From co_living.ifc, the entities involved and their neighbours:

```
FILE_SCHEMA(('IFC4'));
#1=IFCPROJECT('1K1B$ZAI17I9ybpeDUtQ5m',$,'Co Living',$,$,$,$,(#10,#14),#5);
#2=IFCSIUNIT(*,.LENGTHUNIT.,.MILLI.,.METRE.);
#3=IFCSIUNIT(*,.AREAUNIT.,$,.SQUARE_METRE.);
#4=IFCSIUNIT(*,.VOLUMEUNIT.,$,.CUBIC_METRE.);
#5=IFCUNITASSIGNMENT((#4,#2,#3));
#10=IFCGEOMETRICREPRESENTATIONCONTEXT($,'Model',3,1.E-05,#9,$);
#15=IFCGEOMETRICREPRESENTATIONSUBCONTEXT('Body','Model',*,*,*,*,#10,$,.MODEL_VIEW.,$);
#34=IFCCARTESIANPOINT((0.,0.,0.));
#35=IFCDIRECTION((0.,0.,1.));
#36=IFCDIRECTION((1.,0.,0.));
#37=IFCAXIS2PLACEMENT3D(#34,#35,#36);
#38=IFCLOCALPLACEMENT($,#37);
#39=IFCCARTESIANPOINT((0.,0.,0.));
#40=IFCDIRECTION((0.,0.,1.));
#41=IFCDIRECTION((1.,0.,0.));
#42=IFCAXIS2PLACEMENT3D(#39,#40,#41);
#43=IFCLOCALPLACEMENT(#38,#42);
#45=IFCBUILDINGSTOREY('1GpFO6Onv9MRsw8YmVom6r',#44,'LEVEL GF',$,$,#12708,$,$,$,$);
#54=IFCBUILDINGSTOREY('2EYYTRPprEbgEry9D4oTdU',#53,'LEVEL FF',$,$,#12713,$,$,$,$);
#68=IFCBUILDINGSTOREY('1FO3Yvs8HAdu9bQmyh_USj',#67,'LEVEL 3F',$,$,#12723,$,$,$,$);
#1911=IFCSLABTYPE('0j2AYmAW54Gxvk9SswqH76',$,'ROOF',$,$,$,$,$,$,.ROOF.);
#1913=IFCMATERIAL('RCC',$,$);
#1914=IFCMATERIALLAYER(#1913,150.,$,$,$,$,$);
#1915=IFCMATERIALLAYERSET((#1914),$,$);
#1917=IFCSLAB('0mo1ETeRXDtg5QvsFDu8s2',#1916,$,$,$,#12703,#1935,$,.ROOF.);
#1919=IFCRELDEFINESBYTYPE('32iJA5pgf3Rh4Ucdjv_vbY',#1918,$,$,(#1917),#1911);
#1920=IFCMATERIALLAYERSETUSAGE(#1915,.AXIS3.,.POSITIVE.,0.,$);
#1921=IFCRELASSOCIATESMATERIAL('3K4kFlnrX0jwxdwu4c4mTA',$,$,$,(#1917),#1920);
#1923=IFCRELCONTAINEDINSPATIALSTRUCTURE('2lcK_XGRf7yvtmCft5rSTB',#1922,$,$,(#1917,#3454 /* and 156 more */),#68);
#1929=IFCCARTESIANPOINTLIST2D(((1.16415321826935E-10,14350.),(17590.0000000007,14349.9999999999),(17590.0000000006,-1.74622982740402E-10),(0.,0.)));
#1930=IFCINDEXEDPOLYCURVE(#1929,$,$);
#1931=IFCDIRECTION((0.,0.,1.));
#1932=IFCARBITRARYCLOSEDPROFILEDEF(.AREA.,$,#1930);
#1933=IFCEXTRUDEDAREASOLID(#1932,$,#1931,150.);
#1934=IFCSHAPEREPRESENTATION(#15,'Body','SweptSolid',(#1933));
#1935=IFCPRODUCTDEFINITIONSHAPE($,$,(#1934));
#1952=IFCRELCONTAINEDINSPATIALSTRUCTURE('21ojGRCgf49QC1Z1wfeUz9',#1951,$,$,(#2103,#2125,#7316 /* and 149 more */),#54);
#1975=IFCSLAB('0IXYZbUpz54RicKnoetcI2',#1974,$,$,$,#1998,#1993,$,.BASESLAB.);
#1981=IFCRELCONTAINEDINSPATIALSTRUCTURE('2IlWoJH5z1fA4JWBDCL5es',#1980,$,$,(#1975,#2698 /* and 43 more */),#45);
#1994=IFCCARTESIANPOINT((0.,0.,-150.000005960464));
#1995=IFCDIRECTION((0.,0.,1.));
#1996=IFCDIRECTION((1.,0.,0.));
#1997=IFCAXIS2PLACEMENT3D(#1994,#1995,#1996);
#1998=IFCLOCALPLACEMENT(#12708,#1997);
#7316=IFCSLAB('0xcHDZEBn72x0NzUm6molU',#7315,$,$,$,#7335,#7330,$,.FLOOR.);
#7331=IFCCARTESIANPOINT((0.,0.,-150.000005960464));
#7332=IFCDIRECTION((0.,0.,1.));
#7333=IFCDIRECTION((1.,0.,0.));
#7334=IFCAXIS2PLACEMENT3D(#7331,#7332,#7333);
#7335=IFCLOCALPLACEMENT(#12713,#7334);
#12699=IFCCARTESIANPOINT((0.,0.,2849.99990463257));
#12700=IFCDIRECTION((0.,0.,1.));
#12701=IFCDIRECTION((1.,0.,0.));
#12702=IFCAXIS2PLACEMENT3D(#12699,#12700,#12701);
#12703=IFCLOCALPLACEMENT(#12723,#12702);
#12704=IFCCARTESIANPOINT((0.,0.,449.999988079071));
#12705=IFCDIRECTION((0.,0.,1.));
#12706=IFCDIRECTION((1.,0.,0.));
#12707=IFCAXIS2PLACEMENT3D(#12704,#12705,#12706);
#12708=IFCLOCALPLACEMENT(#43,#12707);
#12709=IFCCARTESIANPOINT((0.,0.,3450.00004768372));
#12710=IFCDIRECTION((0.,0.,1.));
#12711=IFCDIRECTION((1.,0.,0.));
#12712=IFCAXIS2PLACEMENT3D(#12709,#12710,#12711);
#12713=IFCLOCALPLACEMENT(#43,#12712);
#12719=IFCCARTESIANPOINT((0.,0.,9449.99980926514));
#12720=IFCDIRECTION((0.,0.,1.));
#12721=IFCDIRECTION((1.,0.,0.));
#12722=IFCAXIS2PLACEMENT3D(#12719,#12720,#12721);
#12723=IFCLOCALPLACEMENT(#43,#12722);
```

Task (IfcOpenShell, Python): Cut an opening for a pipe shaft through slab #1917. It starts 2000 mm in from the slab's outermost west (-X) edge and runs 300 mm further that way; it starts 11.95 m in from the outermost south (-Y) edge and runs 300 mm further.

```python
import numpy as np
import ifcopenshell
import ifcopenshell.api.feature
import ifcopenshell.api.geometry
import ifcopenshell.api.root
import ifcopenshell.geom
import ifcopenshell.util.placement
import ifcopenshell.util.representation
import ifcopenshell.util.shape
import ifcopenshell.util.unit

model = ifcopenshell.open("co_living.ifc")
unit_scale = ifcopenshell.util.unit.calculate_unit_scale(model)
settings = ifcopenshell.geom.settings()


def volume(element):
    """Net volume in cubic metres, openings subtracted."""
    shape = ifcopenshell.geom.create_shape(settings, element)
    return ifcopenshell.util.shape.get_volume(shape.geometry)


slab = model.by_id(1917)
before = volume(slab)

# Extent in the slab's own axes, in metres. The edges named are its -X and -Y sides.
slab_shape = ifcopenshell.geom.create_shape(settings, slab)
vertices = ifcopenshell.util.shape.get_vertices(slab_shape.geometry)
x_min, y_min, bottom = vertices.min(axis=0)
top = vertices[:, 2].max()

opening = ifcopenshell.api.root.create_entity(model, ifc_class="IfcOpeningElement", name="Pipe shaft opening", predefined_type="OPENING")
context = ifcopenshell.util.representation.get_context(model, "Model", "Body", "MODEL_VIEW")
width, depth = 0.3, 0.3
outline = [(0.0, 0.0), (width, 0.0), (width, depth), (0.0, depth), (0.0, 0.0)]
# Overshoot both faces by 50 mm so the cut is clean.
shape = ifcopenshell.api.geometry.add_slab_representation(
    model, context=context, depth=top - bottom + 0.1, polyline=outline
)
ifcopenshell.api.geometry.assign_representation(model, product=opening, representation=shape)

matrix = ifcopenshell.util.placement.get_local_placement(slab.ObjectPlacement)
matrix[:, 3] = matrix @ np.append(np.array([x_min + 2, y_min + 11.95, bottom - 0.05]) / unit_scale, 1.0)
ifcopenshell.api.geometry.edit_object_placement(model, product=opening, matrix=matrix, is_si=False)
ifcopenshell.api.feature.add_feature(model, feature=opening, element=slab)

after = volume(slab)

print(f"slab volume {before:.3f} -> {after:.3f} m3")

model.write("co_living-out.ifc")
```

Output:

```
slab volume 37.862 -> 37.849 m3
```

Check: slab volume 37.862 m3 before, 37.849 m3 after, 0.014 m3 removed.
